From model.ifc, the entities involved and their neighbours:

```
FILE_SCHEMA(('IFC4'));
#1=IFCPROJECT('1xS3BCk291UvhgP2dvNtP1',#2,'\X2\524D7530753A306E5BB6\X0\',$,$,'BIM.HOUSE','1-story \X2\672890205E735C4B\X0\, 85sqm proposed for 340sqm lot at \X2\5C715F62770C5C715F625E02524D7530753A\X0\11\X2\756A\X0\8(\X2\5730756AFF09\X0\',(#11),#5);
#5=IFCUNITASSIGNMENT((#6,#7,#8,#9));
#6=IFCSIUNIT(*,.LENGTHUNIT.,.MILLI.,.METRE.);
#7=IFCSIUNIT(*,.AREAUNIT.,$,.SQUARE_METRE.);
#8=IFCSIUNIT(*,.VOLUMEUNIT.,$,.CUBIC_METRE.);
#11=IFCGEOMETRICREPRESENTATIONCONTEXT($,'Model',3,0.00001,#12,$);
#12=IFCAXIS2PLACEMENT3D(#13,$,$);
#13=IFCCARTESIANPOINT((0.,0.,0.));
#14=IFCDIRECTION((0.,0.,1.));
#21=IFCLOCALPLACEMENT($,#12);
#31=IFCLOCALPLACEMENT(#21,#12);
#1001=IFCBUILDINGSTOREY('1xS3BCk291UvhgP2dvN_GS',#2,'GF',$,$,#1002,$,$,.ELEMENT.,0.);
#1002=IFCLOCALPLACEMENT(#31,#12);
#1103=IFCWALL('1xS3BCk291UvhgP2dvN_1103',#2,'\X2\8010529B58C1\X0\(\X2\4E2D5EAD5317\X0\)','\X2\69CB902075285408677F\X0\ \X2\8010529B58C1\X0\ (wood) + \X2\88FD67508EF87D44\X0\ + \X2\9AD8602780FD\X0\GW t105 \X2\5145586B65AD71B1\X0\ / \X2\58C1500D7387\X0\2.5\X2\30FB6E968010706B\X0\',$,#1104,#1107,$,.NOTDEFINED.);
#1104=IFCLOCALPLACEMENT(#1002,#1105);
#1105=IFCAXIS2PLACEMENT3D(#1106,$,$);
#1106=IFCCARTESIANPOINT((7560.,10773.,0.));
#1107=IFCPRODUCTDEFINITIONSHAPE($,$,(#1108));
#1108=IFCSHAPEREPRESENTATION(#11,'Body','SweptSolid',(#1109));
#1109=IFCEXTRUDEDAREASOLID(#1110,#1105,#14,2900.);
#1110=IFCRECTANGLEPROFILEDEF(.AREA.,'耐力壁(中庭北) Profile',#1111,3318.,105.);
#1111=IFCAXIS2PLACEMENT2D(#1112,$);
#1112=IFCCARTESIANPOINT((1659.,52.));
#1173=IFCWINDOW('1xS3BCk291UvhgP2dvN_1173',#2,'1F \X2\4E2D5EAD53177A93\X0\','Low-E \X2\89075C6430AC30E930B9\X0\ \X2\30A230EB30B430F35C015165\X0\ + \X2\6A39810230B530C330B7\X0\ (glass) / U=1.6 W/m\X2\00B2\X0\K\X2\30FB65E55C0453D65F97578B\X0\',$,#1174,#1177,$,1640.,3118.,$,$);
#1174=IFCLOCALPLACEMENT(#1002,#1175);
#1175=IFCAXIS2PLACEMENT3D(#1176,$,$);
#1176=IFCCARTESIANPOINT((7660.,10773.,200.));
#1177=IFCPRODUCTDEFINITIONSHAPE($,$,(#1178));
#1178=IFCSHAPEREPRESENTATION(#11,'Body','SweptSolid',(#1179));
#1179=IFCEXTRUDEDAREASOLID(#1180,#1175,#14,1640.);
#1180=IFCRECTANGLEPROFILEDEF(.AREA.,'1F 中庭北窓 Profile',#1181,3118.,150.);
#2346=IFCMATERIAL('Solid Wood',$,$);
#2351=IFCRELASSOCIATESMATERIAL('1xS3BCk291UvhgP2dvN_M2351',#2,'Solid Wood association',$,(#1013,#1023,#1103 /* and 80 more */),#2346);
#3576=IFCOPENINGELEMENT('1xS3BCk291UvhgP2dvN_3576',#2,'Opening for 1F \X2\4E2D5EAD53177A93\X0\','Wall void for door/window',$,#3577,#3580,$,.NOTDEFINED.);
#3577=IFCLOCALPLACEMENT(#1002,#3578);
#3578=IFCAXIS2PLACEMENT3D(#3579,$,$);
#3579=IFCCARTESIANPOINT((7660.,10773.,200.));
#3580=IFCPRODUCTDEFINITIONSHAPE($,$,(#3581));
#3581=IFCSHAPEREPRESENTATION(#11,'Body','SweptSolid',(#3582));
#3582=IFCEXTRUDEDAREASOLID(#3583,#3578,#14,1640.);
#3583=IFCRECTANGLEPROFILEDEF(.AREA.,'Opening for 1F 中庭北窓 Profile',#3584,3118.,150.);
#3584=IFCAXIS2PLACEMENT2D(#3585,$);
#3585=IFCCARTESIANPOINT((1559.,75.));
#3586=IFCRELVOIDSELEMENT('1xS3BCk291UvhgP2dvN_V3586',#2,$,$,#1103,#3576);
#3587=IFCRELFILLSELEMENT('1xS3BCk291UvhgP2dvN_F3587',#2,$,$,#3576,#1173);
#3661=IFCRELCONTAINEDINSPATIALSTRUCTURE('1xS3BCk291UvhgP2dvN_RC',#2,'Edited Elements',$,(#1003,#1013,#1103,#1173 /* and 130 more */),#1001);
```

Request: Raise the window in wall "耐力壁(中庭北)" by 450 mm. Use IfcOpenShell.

```python
import numpy as np
import ifcopenshell
import ifcopenshell.api.geometry
import ifcopenshell.util.placement
import ifcopenshell.util.unit

model = ifcopenshell.open("model.ifc")
unit_scale = ifcopenshell.util.unit.calculate_unit_scale(model)

window = model.by_id(1173)
opening = window.FillsVoids[0].RelatingOpeningElement
dz = 450.0

shift = np.array([0.0, 0.0, dz])
# The window is not placed relative to its opening, so move both.
for product in (opening, window):
    matrix = ifcopenshell.util.placement.get_local_placement(product.ObjectPlacement)
    matrix[:3, 3] += shift
    ifcopenshell.api.geometry.edit_object_placement(model, product=product, matrix=matrix, is_si=False)

print(f"moved by {dz * unit_scale:+.3f} m")

model.write("model_rev.ifc")
```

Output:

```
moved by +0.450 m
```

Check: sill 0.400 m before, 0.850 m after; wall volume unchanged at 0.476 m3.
